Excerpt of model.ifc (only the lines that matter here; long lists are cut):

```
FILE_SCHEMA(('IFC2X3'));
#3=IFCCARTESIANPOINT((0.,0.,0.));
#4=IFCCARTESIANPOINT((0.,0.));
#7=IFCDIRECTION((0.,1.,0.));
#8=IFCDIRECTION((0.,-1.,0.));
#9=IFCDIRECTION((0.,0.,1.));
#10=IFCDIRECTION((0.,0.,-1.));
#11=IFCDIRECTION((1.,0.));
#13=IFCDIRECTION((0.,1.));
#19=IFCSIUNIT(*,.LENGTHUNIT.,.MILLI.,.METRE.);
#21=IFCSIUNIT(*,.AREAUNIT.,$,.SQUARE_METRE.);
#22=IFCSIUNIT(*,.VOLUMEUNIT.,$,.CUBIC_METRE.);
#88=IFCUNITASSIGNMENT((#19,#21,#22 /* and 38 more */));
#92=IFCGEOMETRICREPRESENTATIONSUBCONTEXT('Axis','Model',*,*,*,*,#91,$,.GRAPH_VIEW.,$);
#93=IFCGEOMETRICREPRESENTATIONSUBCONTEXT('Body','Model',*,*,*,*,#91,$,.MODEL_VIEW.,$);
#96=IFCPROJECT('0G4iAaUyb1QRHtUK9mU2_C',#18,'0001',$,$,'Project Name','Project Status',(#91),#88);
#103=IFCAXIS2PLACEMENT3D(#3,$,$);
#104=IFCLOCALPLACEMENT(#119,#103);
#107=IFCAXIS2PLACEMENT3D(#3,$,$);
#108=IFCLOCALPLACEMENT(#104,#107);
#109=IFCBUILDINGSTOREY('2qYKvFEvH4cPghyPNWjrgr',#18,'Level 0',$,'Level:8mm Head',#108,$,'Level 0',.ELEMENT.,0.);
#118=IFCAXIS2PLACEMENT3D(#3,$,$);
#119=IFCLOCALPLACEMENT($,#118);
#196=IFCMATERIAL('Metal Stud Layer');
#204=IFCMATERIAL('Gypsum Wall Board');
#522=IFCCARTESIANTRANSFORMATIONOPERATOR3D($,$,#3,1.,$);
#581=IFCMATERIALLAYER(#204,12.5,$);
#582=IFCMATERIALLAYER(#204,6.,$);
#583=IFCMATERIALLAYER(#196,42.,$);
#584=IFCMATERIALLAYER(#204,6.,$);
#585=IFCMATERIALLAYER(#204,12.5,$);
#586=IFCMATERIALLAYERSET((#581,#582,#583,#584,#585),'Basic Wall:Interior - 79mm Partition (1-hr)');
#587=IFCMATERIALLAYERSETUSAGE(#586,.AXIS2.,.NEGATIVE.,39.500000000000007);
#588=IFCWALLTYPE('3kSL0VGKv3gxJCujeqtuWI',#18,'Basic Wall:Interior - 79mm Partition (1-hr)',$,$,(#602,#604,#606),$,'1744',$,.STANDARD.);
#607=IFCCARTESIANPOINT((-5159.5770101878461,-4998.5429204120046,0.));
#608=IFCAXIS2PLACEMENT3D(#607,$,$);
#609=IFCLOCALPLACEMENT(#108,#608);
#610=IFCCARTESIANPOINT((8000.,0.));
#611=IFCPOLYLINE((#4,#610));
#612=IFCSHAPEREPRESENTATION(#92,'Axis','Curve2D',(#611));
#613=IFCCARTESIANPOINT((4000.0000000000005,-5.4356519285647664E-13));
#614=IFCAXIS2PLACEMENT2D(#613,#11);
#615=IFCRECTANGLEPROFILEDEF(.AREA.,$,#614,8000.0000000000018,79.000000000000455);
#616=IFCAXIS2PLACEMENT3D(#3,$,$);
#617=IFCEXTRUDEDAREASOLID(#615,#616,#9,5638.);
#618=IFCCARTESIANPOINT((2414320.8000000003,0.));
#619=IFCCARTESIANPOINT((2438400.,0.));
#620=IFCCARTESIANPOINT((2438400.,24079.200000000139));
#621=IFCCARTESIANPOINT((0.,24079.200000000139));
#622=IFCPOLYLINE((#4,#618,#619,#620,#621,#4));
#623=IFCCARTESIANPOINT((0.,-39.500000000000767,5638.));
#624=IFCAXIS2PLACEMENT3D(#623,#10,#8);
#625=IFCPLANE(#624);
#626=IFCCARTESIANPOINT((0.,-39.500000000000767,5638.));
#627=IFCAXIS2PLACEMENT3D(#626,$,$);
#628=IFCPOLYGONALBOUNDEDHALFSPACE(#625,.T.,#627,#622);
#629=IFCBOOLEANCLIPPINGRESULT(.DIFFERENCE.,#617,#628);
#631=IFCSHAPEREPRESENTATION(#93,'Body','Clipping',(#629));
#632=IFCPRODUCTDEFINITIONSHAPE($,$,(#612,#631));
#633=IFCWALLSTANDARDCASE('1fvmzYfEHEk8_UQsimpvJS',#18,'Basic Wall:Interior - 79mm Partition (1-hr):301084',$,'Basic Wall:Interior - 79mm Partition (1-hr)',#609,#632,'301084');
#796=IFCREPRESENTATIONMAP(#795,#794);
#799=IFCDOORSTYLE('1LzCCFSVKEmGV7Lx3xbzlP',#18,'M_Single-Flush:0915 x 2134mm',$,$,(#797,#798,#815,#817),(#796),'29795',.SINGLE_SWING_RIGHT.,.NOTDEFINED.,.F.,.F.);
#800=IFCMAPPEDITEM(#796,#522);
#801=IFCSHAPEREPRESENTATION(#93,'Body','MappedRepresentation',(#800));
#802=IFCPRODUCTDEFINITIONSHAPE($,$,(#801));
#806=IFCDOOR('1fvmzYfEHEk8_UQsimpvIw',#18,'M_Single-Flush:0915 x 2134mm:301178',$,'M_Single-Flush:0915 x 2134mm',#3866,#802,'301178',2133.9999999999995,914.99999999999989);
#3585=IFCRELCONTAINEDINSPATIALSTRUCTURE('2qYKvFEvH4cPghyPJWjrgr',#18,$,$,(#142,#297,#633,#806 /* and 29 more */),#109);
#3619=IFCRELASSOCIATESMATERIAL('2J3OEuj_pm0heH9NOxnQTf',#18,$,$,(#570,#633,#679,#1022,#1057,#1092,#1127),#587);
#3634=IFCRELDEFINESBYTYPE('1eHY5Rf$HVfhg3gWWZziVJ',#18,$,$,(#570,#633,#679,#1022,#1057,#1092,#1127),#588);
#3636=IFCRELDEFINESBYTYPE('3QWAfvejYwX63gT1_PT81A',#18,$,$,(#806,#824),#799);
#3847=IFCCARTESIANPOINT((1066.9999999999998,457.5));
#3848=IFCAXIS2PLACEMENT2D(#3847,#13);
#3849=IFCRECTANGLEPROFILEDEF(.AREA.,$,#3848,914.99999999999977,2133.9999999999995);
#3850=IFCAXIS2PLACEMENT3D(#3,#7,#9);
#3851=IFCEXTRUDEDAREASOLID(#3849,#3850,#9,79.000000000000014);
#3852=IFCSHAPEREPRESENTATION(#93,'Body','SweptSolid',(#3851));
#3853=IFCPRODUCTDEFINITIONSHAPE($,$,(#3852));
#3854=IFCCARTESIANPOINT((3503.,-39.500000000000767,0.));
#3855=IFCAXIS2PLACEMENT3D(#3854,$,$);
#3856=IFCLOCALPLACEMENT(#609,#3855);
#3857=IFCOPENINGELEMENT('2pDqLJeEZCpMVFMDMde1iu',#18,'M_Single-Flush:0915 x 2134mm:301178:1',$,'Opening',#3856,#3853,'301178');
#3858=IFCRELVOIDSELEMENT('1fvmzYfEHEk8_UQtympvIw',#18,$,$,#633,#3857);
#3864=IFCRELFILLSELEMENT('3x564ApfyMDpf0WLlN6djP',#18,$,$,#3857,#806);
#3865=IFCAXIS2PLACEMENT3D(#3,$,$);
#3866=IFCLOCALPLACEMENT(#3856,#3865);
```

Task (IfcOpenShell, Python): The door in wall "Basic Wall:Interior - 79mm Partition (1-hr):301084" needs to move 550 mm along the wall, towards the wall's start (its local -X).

```python
import ifcopenshell
import ifcopenshell.api.geometry
import ifcopenshell.util.placement
import ifcopenshell.util.unit

model = ifcopenshell.open("model.ifc")
unit_scale = ifcopenshell.util.unit.calculate_unit_scale(model)

door = model.by_guid("1fvmzYfEHEk8_UQsimpvIw")
opening = door.FillsVoids[0].RelatingOpeningElement
wall = opening.VoidsElements[0].RelatingBuildingElement

wall_matrix = ifcopenshell.util.placement.get_local_placement(wall.ObjectPlacement)
shift = wall_matrix[:3, 0] * -0.55 / unit_scale
before = ifcopenshell.util.placement.get_local_placement(door.ObjectPlacement)[:3, 3].copy()

# The door is placed relative to its opening, so it follows when the opening moves.
matrix = ifcopenshell.util.placement.get_local_placement(opening.ObjectPlacement)
matrix[:3, 3] += shift
ifcopenshell.api.geometry.edit_object_placement(
    model, product=opening, matrix=matrix, is_si=False, should_transform_children=True
)

after = ifcopenshell.util.placement.get_local_placement(door.ObjectPlacement)[:3, 3]
print("door moved by", (after - before).round(3) + 0.0)

model.write("model-out.ifc")
```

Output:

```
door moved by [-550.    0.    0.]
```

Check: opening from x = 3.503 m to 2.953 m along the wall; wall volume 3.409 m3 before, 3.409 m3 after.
